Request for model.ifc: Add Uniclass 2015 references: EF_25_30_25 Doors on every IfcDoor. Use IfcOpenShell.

First a look at what the model holds.

```python
import ifcopenshell

model = ifcopenshell.open("model.ifc")
print(model.schema)
print("classifications:", [c.Name for c in model.by_type("IfcClassification")])
for ifc_class in ("IfcDoor", "IfcRoof", "IfcStair", "IfcWall", "IfcWindow"):
    print(ifc_class, len(model.by_type(ifc_class)))
```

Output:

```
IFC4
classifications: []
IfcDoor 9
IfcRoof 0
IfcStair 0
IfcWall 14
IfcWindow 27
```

```python
import ifcopenshell
import ifcopenshell.api.classification

model = ifcopenshell.open("model.ifc")

system = ifcopenshell.api.classification.add_classification(model, classification="Uniclass 2015")

codes = {
    "IfcDoor": ("EF_25_30_25", "Doors"),
}
for ifc_class, (code, name) in codes.items():
    products = model.by_type(ifc_class)
    ifcopenshell.api.classification.add_reference(
        model, products=products, classification=system, identification=code, name=name
    )
    print(code, len(products))

model.write("model_updated.ifc")
```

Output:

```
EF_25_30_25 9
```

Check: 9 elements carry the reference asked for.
